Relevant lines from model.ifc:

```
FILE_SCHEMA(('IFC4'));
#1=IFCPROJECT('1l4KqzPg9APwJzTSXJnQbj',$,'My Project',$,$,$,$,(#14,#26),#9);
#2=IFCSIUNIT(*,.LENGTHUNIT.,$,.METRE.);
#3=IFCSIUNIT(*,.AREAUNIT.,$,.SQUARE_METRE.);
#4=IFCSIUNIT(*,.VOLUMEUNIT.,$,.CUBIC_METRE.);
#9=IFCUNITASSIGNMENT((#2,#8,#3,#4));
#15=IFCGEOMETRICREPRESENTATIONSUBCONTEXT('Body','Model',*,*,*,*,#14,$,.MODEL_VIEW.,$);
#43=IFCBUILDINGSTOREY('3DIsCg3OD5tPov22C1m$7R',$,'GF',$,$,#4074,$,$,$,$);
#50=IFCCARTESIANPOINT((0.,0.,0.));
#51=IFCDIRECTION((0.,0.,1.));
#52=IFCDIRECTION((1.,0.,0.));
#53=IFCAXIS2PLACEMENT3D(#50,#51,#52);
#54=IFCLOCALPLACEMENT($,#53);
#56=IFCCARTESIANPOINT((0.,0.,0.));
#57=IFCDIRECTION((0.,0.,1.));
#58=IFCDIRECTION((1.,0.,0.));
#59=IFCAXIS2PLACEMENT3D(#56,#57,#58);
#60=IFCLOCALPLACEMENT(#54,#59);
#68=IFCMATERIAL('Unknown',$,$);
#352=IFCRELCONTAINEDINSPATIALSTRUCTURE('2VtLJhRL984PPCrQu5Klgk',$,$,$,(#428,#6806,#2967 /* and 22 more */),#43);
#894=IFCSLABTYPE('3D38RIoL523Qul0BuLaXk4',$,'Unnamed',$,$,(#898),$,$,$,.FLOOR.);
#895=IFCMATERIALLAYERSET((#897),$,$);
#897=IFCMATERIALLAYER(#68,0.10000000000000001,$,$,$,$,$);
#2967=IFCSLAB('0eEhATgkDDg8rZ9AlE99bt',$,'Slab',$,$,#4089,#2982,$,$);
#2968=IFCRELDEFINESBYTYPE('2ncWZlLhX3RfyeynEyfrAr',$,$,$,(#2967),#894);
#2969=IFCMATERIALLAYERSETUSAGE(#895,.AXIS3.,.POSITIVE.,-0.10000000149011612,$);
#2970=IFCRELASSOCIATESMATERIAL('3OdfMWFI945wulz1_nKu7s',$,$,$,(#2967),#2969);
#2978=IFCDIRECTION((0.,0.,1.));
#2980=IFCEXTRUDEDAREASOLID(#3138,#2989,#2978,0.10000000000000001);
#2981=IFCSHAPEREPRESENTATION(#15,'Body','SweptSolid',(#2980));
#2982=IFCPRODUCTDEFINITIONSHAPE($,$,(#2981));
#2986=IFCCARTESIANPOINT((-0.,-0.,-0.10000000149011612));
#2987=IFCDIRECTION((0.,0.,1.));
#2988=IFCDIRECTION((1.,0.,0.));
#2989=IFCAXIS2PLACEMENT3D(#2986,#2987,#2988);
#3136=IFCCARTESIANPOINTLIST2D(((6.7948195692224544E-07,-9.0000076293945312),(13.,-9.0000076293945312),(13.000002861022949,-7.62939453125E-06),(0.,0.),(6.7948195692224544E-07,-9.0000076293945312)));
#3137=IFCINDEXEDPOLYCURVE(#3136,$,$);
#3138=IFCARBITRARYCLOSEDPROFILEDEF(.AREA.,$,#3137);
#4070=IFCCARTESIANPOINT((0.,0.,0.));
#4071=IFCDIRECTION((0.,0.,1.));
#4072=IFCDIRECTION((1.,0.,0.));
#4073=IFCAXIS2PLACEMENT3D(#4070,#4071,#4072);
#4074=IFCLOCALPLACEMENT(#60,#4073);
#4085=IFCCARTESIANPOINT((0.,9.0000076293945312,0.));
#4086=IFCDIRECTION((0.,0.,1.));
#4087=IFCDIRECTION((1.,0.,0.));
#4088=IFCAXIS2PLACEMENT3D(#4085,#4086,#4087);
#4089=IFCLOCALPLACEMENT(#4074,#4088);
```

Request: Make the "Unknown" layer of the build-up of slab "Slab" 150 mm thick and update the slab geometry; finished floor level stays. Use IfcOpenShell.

```python
import ifcopenshell
import ifcopenshell.util.element
import ifcopenshell.util.representation

model = ifcopenshell.open("model.ifc")

layer_set = model.by_id(895)
layer = next(l for l in layer_set.MaterialLayers if l.Material and l.Material.Name == "Unknown")
change = 0.15 - layer.LayerThickness
layer.LayerThickness += change

# Geometry does not follow the layer set by itself.
slabs = [e for e in ifcopenshell.util.element.get_elements_by_material(model, layer_set) if e.is_a("IfcSlab")]
for slab in sorted(slabs, key=lambda e: e.id()):
    body = ifcopenshell.util.representation.get_representation(slab, "Model", "Body")
    solid = body.Items[0]
    old_depth = solid.Depth
    solid.Depth += change
    # Extruded upwards: lower the start of the extrusion so the top stays.
    x, y, z = solid.Position.Location.Coordinates
    solid.Position.Location = model.createIfcCartesianPoint((x, y, z - change))
    print(slab.id(), f"{old_depth:g} -> {solid.Depth:g}")

# The layers are counted up from the underside, which has moved.
for usage in {ifcopenshell.util.element.get_material(slab) for slab in slabs}:
    usage.OffsetFromReferenceLine -= change

model.write("model_updated.ifc")
```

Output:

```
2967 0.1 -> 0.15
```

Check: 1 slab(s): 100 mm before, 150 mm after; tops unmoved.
